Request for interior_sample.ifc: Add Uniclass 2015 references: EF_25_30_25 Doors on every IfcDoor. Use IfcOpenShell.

First a look at what the model holds.

```python
import ifcopenshell

model = ifcopenshell.open("interior_sample.ifc")
print(model.schema)
print("classifications:", [c.Name for c in model.by_type("IfcClassification")])
for ifc_class in ("IfcDoor", "IfcRoof", "IfcStair", "IfcWall", "IfcWindow"):
    print(ifc_class, len(model.by_type(ifc_class)))
```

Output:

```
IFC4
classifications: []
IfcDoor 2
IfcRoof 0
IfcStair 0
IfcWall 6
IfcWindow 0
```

```python
import ifcopenshell
import ifcopenshell.api.classification

model = ifcopenshell.open("interior_sample.ifc")

system = ifcopenshell.api.classification.add_classification(model, classification="Uniclass 2015")

codes = {
    "IfcDoor": ("EF_25_30_25", "Doors"),
}
for ifc_class, (code, name) in codes.items():
    products = model.by_type(ifc_class)
    ifcopenshell.api.classification.add_reference(
        model, products=products, classification=system, identification=code, name=name
    )
    print(code, len(products))

model.write("interior_sample_edited.ifc")
```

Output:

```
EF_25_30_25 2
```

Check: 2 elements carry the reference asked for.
